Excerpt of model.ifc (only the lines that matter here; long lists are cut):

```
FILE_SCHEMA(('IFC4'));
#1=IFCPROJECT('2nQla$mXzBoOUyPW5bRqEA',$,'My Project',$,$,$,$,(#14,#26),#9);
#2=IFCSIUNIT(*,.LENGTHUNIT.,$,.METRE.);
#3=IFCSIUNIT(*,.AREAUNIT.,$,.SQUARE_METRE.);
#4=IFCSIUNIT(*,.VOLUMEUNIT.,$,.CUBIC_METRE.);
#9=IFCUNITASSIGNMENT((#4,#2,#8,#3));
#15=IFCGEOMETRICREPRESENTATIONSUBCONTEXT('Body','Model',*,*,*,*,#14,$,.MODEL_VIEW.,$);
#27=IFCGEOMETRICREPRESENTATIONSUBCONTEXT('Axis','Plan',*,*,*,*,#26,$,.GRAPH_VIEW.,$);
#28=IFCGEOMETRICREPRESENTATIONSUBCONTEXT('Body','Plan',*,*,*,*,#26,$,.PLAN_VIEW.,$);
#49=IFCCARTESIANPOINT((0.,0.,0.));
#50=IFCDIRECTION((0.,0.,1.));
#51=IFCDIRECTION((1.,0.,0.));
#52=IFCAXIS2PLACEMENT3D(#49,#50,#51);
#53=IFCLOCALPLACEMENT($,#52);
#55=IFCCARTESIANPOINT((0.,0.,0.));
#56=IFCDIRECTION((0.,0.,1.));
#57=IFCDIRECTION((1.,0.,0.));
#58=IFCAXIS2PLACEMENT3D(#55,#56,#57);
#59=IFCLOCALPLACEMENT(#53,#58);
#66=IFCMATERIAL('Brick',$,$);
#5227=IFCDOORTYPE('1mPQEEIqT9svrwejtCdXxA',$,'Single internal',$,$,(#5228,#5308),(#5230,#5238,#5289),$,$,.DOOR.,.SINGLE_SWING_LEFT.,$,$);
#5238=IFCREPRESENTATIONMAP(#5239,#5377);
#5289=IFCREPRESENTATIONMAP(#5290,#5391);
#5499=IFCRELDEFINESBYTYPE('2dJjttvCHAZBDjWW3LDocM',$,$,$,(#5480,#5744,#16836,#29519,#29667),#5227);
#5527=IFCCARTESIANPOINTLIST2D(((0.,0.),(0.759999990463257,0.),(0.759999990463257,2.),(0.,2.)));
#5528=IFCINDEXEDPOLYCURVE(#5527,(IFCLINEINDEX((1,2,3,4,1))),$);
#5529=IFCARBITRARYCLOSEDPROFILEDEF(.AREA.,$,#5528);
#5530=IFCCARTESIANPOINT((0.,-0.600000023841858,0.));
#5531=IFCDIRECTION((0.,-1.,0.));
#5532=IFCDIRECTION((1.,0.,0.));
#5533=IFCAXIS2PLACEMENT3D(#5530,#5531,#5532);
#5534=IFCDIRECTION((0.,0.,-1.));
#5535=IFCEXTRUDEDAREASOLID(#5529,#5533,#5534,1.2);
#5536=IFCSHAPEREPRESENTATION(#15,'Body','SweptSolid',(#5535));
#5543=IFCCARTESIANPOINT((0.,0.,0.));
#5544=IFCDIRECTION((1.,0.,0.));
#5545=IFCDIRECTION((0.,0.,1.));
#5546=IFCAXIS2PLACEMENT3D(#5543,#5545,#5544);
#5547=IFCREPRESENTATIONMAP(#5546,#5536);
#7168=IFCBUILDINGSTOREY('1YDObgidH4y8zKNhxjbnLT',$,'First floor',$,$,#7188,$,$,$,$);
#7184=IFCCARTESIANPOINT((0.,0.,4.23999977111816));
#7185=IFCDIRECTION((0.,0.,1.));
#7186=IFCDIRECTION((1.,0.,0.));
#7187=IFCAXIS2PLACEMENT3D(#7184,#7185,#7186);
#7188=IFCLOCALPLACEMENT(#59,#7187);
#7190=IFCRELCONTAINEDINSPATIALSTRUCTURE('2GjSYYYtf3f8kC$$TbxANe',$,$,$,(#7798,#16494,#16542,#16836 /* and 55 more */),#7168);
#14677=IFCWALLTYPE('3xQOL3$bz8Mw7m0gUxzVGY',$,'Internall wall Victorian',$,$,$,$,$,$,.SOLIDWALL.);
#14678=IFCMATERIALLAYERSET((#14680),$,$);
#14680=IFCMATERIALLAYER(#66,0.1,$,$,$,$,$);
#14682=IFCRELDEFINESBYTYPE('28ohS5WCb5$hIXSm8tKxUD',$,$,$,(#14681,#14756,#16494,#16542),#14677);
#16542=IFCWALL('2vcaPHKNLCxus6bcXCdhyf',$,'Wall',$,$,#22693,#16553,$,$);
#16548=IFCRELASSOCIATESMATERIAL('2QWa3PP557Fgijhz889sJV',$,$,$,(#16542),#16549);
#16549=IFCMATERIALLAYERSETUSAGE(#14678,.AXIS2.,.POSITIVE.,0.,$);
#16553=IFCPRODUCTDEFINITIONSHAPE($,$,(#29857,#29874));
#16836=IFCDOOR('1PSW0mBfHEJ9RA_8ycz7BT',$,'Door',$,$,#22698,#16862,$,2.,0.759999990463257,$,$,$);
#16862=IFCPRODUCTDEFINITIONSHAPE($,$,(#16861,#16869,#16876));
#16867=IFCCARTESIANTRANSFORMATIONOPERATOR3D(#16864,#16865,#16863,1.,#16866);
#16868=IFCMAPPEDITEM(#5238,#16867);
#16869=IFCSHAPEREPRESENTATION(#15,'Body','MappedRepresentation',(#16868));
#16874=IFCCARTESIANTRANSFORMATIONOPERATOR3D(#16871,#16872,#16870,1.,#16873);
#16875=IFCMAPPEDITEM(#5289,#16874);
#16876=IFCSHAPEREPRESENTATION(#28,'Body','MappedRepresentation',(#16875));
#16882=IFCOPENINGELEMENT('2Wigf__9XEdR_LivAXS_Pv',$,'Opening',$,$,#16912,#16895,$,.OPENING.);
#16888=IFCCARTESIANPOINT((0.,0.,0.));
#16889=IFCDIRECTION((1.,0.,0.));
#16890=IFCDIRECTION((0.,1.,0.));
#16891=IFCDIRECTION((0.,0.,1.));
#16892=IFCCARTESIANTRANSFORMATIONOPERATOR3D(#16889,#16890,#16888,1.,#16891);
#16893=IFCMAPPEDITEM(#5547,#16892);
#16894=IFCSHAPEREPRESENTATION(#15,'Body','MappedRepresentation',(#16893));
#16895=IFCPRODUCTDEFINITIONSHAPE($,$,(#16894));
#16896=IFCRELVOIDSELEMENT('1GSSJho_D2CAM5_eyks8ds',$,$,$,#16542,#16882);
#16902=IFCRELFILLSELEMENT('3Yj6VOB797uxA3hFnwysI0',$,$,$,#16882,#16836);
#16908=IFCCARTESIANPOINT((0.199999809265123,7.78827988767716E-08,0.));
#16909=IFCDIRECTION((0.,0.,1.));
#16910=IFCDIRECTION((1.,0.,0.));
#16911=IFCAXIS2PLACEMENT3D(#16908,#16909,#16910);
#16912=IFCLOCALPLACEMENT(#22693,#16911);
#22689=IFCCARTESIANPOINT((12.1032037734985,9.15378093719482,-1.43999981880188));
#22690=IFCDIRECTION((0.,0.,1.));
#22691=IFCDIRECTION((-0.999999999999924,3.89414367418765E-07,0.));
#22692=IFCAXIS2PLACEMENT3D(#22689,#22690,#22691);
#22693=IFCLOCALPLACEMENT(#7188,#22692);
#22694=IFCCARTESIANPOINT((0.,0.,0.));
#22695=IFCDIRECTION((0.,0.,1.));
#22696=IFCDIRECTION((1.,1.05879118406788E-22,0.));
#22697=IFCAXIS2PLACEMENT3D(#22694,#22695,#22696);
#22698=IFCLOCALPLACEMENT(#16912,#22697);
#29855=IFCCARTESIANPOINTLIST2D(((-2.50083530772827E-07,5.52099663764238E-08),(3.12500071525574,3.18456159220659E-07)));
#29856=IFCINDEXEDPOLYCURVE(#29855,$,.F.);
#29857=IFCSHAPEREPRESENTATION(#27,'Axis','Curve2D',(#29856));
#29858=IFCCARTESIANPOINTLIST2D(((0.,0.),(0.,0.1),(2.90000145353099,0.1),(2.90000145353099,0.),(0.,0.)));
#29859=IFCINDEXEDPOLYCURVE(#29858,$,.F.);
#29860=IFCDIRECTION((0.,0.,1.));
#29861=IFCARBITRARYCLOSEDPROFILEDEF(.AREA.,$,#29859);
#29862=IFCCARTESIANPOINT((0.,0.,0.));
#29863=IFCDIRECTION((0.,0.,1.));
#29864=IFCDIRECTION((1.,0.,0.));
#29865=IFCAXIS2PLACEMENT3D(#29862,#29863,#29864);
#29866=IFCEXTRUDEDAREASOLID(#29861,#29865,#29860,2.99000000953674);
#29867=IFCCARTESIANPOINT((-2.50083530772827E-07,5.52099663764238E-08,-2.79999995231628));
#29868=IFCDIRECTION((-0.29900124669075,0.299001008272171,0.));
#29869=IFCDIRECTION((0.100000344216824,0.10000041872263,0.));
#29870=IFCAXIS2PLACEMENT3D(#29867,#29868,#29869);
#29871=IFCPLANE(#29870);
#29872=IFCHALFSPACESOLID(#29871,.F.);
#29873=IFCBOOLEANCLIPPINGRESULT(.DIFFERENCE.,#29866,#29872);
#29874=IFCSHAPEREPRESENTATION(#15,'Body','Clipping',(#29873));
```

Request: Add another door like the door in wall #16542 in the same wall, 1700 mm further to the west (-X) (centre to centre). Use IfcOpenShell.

```python
import ifcopenshell
import ifcopenshell.api.feature
import ifcopenshell.api.geometry
import ifcopenshell.api.root
import ifcopenshell.geom
import ifcopenshell.util.element
import ifcopenshell.util.placement
import ifcopenshell.util.shape
import ifcopenshell.util.unit

model = ifcopenshell.open("model.ifc")
unit_scale = ifcopenshell.util.unit.calculate_unit_scale(model)
settings = ifcopenshell.geom.settings()


def volume(element):
    """Net volume in cubic metres, openings subtracted."""
    shape = ifcopenshell.geom.create_shape(settings, element)
    return ifcopenshell.util.shape.get_volume(shape.geometry)


door = model.by_guid("1PSW0mBfHEJ9RA_8ycz7BT")
opening = door.FillsVoids[0].RelatingOpeningElement
wall = opening.VoidsElements[0].RelatingBuildingElement
before = volume(wall)
shift = ifcopenshell.util.placement.get_local_placement(wall.ObjectPlacement)[:3, 0] * 1.7 / unit_scale

# copy_class copies the void relationship, type, container and properties, but no geometry.
new_opening = ifcopenshell.api.root.copy_class(model, product=opening)
new_opening.Representation = ifcopenshell.util.element.copy_deep(
    model, opening.Representation, exclude=["IfcGeometricRepresentationContext", "IfcRepresentationMap"]
)
new_door = ifcopenshell.api.root.copy_class(model, product=door)
new_door.Representation = ifcopenshell.util.element.copy_deep(
    model, door.Representation, exclude=["IfcGeometricRepresentationContext", "IfcRepresentationMap"]
)
ifcopenshell.api.feature.add_filling(model, opening=new_opening, element=new_door)

for old, new in ((opening, new_opening), (door, new_door)):
    matrix = ifcopenshell.util.placement.get_local_placement(old.ObjectPlacement)
    matrix[:3, 3] += shift
    ifcopenshell.api.geometry.edit_object_placement(model, product=new, matrix=matrix, is_si=False)

after = volume(wall)

print(f"wall volume {before:.3f} -> {after:.3f} m3")

model.write("model_v2.ifc")
```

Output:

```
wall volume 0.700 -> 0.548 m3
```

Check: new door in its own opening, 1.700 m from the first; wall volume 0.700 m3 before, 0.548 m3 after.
